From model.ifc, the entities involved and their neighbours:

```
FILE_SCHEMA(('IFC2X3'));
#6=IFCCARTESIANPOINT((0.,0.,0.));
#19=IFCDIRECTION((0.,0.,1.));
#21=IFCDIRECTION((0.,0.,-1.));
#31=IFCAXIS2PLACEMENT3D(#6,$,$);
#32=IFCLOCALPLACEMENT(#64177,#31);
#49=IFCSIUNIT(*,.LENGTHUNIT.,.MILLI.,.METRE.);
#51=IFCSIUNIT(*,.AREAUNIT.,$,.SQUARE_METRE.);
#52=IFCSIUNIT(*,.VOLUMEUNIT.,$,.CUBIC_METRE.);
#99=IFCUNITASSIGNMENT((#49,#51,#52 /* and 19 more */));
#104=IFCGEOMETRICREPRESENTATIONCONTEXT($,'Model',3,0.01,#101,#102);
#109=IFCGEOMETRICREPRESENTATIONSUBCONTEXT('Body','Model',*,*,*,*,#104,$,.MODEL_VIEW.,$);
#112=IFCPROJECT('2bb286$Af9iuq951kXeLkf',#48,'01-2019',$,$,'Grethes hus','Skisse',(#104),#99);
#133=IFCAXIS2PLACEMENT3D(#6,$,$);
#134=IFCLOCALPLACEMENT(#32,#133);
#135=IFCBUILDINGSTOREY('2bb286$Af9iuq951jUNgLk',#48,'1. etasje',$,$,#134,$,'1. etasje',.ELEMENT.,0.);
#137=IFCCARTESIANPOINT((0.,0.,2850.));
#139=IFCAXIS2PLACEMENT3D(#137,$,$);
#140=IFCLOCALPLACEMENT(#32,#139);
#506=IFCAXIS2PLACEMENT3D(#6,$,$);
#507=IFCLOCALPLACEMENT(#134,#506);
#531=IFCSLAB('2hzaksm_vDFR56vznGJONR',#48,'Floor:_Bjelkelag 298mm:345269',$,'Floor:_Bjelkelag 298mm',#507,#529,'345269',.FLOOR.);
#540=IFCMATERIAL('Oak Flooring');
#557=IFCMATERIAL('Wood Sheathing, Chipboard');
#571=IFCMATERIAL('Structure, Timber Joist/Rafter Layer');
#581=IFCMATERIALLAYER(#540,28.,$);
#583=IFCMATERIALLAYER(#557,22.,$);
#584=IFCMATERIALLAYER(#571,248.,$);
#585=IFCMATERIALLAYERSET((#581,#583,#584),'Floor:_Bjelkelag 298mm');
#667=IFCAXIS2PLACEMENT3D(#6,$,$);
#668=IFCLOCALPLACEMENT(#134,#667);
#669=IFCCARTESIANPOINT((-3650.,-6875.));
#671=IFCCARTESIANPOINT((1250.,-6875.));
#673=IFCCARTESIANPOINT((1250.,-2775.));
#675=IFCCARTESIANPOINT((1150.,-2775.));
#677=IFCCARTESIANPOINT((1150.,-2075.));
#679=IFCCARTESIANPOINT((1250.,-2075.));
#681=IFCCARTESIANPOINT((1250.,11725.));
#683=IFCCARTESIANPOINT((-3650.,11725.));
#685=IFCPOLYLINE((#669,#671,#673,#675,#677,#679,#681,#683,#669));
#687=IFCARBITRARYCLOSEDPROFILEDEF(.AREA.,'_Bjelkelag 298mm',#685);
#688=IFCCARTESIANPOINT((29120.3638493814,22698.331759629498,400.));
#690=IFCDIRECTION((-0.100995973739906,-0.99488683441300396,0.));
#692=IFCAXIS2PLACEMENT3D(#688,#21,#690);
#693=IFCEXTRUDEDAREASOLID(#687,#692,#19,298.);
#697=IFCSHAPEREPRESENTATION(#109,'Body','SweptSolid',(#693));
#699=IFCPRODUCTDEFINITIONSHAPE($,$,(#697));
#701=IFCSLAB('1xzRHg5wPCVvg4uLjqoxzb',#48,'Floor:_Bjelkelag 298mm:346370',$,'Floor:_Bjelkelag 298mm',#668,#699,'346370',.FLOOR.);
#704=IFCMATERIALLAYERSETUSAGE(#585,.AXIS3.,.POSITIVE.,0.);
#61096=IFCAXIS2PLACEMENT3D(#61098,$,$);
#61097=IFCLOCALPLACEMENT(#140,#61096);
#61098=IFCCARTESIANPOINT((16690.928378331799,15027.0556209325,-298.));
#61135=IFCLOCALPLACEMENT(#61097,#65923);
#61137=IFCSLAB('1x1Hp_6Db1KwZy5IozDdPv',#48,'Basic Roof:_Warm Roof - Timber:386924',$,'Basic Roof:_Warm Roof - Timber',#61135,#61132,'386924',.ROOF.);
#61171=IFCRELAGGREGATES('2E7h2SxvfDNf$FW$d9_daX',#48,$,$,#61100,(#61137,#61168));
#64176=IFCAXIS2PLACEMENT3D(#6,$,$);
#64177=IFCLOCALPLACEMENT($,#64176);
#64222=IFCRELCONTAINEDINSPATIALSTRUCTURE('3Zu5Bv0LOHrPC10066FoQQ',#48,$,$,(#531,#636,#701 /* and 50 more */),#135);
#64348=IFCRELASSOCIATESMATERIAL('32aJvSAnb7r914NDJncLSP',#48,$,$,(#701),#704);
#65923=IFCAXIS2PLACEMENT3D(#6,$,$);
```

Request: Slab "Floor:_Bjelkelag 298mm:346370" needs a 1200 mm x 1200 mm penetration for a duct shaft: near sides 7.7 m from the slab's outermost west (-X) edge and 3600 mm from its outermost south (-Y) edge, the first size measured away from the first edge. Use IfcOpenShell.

```python
import numpy as np
import ifcopenshell
import ifcopenshell.api.feature
import ifcopenshell.api.geometry
import ifcopenshell.api.root
import ifcopenshell.geom
import ifcopenshell.util.placement
import ifcopenshell.util.representation
import ifcopenshell.util.shape
import ifcopenshell.util.unit

model = ifcopenshell.open("model.ifc")
unit_scale = ifcopenshell.util.unit.calculate_unit_scale(model)
settings = ifcopenshell.geom.settings()


def volume(element):
    """Net volume in cubic metres, openings subtracted."""
    shape = ifcopenshell.geom.create_shape(settings, element)
    return ifcopenshell.util.shape.get_volume(shape.geometry)


slab = model.by_id(701)
before = volume(slab)

# Extent in the slab's own axes, in metres. The edges named are its -X and -Y sides.
slab_shape = ifcopenshell.geom.create_shape(settings, slab)
vertices = ifcopenshell.util.shape.get_vertices(slab_shape.geometry)
x_min, y_min, bottom = vertices.min(axis=0)
top = vertices[:, 2].max()

opening = ifcopenshell.api.root.create_entity(model, ifc_class="IfcOpeningElement", name="Duct shaft opening")
context = ifcopenshell.util.representation.get_context(model, "Model", "Body", "MODEL_VIEW")
width, depth = 1.2, 1.2
outline = [(0.0, 0.0), (width, 0.0), (width, depth), (0.0, depth), (0.0, 0.0)]
# Overshoot both faces by 50 mm so the cut is clean.
shape = ifcopenshell.api.geometry.add_slab_representation(
    model, context=context, depth=top - bottom + 0.1, polyline=outline
)
ifcopenshell.api.geometry.assign_representation(model, product=opening, representation=shape)

matrix = ifcopenshell.util.placement.get_local_placement(slab.ObjectPlacement)
matrix[:, 3] = matrix @ np.append(np.array([x_min + 7.7, y_min + 3.6, bottom - 0.05]) / unit_scale, 1.0)
ifcopenshell.api.geometry.edit_object_placement(model, product=opening, matrix=matrix, is_si=False)
ifcopenshell.api.feature.add_feature(model, feature=opening, element=slab)

after = volume(slab)

print(f"slab volume {before:.3f} -> {after:.3f} m3")

model.write("model-out.ifc")
```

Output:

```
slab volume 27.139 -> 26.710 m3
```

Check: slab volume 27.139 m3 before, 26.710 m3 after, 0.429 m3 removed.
